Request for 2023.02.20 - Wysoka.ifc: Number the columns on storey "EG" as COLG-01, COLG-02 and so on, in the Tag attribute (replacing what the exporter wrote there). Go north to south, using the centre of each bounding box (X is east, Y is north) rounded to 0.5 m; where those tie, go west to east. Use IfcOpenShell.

First a look at what the model holds.

```python
import ifcopenshell
import ifcopenshell.util.element
import ifcopenshell.util.placement

model = ifcopenshell.open("2023.02.20 - Wysoka.ifc")
print(model.schema)
storey = next(s for s in model.by_type("IfcBuildingStorey") if s.Name == "EG")
columns = [e for e in ifcopenshell.util.element.get_decomposition(storey) if e.is_a("IfcColumn")]
for e in sorted(columns, key=lambda e: e.id()):
    origin = ifcopenshell.util.placement.get_local_placement(e.ObjectPlacement)[:3, 3]
    print(e.id(), e.Tag, e.Name, origin.round(2) + 0.0, sep=" | ")
```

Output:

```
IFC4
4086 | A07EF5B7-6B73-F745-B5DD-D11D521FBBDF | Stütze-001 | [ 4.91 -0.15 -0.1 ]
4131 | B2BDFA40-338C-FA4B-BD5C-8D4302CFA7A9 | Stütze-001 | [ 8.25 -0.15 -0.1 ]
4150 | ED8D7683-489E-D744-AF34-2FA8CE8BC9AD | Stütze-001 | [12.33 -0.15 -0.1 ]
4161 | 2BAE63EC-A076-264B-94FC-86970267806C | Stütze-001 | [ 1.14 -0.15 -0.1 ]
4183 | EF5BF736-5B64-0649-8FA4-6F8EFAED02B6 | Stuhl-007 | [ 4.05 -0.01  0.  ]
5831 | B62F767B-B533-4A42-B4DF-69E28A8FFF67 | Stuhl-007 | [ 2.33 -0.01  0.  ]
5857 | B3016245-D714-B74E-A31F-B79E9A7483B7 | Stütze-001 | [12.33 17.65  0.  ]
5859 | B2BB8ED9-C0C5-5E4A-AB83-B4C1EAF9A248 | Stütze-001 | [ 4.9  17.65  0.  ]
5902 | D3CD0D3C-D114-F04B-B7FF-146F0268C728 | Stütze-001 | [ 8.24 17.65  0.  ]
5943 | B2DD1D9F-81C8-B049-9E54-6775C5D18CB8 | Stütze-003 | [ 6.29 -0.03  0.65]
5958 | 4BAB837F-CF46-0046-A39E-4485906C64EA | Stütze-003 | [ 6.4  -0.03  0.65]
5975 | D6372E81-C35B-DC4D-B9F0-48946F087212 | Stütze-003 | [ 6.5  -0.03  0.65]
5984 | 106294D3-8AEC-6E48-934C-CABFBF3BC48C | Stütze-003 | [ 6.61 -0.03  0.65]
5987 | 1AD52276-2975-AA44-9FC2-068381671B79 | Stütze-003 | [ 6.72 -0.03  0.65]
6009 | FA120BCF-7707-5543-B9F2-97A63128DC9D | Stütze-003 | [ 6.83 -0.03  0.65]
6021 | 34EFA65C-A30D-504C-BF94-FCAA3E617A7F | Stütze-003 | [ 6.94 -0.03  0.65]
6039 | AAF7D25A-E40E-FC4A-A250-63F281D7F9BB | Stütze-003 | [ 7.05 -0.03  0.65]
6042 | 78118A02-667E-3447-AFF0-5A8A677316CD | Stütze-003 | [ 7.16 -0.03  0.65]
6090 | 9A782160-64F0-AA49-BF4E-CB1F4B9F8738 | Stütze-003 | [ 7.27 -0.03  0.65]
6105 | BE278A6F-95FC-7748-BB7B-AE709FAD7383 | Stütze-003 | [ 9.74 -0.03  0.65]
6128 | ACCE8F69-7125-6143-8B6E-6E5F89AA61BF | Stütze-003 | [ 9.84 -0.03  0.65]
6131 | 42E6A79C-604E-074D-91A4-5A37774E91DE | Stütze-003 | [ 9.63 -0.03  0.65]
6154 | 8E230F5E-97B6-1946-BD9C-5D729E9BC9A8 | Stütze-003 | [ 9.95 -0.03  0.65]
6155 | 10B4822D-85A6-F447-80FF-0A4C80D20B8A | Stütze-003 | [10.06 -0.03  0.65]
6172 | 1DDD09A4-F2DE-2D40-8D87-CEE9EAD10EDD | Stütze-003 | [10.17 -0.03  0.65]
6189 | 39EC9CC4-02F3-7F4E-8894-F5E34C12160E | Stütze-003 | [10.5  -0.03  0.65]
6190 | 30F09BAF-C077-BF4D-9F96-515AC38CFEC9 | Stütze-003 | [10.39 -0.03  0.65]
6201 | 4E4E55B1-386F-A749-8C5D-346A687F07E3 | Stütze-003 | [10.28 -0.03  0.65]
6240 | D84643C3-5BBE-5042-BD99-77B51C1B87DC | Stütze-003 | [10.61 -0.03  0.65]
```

```python
import ifcopenshell
import ifcopenshell.geom
import ifcopenshell.util.element
import ifcopenshell.util.shape

model = ifcopenshell.open("2023.02.20 - Wysoka.ifc")
settings = ifcopenshell.geom.settings()
settings.set("use-world-coords", True)


def centre(element):
    shape = ifcopenshell.geom.create_shape(settings, element)
    return ifcopenshell.util.shape.get_bbox_centroid(shape.geometry)


storey = next(s for s in model.by_type("IfcBuildingStorey") if s.Name == "EG")
columns = [e for e in ifcopenshell.util.element.get_decomposition(storey) if e.is_a("IfcColumn")]

# Insertion points can sit at a corner or the storey origin, so sort by the geometry (in metres).
centres = {e: centre(e) for e in columns}
columns.sort(key=lambda e: (-round(centres[e][1] / 0.5), centres[e][0]))

for i, e in enumerate(columns, start=1):
    number = f"COLG-{i:02d}"
    e.Tag = number
    print(e.id(), number)

model.write("2023.02.20 - Wysoka_updated.ifc")
```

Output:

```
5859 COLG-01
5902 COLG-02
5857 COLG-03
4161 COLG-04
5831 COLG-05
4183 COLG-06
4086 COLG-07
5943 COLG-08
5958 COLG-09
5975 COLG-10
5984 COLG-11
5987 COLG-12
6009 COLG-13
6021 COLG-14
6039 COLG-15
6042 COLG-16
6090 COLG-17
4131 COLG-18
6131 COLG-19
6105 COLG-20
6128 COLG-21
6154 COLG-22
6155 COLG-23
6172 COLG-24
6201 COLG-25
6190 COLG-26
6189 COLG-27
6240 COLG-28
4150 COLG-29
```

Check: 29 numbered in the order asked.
